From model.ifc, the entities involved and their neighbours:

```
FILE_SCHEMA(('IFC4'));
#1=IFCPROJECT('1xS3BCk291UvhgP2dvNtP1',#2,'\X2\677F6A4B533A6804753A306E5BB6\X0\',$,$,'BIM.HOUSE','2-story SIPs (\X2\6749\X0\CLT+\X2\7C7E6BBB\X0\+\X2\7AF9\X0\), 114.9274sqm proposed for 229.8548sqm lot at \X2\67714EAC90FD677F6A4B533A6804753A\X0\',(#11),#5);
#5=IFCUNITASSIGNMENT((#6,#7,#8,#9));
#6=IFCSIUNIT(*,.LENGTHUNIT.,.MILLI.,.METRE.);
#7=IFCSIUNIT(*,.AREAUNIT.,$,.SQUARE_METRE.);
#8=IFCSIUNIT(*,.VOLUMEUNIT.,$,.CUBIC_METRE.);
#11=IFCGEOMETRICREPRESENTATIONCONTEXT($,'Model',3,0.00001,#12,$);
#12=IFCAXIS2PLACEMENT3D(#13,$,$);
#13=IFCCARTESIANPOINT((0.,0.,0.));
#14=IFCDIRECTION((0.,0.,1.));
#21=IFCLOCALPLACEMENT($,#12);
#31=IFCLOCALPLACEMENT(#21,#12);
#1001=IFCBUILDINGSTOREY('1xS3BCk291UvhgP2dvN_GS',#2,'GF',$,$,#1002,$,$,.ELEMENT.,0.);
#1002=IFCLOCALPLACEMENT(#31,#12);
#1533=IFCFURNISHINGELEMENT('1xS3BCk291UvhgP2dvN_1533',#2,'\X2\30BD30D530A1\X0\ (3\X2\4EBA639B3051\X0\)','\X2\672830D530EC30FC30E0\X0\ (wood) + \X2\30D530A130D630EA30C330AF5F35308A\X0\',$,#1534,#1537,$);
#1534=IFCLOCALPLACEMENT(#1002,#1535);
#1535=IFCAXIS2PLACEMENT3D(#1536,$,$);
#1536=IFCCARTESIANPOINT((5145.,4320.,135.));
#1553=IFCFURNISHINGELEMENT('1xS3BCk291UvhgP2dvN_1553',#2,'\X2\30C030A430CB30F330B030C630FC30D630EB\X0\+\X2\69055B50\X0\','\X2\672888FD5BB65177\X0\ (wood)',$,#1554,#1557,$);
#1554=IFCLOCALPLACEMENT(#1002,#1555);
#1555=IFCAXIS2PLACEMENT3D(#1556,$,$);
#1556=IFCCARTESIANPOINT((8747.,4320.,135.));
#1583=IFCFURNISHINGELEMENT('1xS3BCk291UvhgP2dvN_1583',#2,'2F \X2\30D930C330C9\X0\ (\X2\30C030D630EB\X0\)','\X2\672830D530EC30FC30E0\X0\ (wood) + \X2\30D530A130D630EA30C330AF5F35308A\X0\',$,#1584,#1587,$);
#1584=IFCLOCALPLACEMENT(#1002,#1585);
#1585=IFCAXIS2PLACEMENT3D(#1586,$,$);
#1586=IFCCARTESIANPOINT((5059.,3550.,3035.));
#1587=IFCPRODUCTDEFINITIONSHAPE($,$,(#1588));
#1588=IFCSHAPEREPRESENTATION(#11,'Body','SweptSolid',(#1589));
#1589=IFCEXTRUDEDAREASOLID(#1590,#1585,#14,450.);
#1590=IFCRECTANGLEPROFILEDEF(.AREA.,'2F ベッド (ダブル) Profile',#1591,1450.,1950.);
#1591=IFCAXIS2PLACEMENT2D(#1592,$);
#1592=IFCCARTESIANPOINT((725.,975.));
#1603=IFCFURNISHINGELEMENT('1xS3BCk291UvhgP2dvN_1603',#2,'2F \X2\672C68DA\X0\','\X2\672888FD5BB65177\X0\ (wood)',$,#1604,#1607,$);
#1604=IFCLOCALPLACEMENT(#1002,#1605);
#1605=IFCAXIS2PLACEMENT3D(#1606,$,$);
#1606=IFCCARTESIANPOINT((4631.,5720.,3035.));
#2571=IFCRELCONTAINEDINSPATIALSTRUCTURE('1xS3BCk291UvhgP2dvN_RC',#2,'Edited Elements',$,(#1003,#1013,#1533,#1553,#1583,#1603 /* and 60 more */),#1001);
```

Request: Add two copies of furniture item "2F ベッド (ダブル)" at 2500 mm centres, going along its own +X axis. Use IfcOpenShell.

```python
import ifcopenshell
import ifcopenshell.api.geometry
import ifcopenshell.api.root
import ifcopenshell.util.element
import ifcopenshell.util.placement

model = ifcopenshell.open("model.ifc")


def reuse_history(source, copy):
    """copy_class also copies each property set's owner history, people and application; keep the originals."""
    for rel in copy.IsDefinedBy:
        if rel.is_a("IfcRelDefinesByProperties") and (history := rel.RelatingPropertyDefinition.OwnerHistory):
            rel.RelatingPropertyDefinition.OwnerHistory = source.OwnerHistory
            ifcopenshell.util.element.remove_deep2(model, history)


source = model.by_id(1583)
base = ifcopenshell.util.placement.get_local_placement(source.ObjectPlacement)
step = base[:3, 0] * 2500.0

for i in range(1, 3):
    copy = ifcopenshell.api.root.copy_class(model, product=source)
    copy.Representation = ifcopenshell.util.element.copy_deep(
        model, source.Representation, exclude=["IfcGeometricRepresentationContext", "IfcRepresentationMap"]
    )
    reuse_history(source, copy)
    matrix = base.copy()
    matrix[:3, 3] += i * step
    print("added at", matrix[:3, 3].round(3) + 0.0)
    ifcopenshell.api.geometry.edit_object_placement(model, product=copy, matrix=matrix, is_si=False)

model.write("model_updated.ifc")
```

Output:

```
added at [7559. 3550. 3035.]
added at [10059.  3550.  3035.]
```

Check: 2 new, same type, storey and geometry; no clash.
